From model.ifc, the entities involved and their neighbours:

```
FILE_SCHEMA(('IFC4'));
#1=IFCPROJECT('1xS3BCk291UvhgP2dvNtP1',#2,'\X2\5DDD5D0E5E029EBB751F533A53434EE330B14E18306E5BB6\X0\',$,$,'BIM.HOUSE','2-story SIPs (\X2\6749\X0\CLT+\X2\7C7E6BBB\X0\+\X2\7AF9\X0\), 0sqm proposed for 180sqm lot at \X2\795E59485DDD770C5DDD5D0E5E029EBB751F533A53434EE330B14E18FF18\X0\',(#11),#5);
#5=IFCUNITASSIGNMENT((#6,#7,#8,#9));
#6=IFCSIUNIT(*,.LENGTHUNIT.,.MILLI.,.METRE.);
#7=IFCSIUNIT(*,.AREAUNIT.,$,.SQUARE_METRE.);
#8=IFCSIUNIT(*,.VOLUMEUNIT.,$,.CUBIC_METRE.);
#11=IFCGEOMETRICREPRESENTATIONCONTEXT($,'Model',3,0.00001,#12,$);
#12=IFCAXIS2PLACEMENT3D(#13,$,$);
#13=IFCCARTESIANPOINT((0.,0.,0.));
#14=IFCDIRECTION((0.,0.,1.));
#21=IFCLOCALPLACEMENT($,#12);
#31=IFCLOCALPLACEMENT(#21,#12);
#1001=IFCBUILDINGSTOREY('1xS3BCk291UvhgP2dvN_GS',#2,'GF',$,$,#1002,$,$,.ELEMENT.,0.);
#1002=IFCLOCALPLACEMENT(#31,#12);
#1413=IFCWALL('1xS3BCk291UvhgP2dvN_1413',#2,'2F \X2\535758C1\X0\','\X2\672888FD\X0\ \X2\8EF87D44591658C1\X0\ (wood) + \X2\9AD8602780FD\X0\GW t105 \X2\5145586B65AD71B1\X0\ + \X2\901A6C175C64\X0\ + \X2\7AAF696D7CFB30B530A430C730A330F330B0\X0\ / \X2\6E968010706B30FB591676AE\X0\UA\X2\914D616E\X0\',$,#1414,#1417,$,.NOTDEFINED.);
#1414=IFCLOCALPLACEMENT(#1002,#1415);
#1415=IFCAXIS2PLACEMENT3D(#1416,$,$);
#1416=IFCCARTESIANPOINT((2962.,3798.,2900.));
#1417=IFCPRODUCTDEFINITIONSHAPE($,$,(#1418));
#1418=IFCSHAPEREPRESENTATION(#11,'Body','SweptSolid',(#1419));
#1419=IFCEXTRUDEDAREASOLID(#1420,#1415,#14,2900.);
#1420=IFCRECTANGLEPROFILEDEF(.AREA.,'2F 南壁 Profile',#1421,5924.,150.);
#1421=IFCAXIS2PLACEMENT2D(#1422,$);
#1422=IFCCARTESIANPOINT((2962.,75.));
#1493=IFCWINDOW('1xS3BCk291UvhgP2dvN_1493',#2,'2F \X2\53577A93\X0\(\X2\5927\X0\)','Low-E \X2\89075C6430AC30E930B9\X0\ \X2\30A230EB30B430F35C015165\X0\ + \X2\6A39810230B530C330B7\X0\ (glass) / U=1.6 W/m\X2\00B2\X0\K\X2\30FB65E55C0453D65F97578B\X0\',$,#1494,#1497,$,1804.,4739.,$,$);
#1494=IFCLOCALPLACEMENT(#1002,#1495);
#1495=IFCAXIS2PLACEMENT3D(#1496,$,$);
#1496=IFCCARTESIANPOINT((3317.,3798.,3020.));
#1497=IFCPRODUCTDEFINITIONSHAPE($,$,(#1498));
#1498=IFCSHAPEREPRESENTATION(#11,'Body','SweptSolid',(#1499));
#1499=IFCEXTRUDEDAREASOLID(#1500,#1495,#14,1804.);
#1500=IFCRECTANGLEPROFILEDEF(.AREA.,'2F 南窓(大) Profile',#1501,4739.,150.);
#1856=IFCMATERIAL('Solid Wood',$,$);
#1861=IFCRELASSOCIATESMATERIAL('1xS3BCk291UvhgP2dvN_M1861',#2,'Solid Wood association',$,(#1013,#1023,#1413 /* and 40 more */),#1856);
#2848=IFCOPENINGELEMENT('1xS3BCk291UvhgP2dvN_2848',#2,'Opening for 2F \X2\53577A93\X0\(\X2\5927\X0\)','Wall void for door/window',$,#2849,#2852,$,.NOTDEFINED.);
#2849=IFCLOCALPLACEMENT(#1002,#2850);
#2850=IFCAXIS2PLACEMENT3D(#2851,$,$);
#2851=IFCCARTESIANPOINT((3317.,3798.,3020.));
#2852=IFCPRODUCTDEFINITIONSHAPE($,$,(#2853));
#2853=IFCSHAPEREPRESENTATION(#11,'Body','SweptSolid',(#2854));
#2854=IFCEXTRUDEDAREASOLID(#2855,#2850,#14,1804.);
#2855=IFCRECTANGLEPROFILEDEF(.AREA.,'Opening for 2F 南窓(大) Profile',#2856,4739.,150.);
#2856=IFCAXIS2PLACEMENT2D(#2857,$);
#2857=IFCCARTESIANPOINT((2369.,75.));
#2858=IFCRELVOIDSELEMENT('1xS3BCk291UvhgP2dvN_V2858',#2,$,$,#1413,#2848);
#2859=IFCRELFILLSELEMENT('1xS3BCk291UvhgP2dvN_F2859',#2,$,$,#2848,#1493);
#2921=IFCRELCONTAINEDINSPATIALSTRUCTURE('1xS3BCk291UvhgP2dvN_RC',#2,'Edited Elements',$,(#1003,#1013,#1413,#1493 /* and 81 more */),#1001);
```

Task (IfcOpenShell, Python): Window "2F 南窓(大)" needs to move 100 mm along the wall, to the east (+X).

```python
import ifcopenshell
import ifcopenshell.api.geometry
import ifcopenshell.util.placement
import ifcopenshell.util.unit

model = ifcopenshell.open("model.ifc")
unit_scale = ifcopenshell.util.unit.calculate_unit_scale(model)

window = model.by_guid("1xS3BCk291UvhgP2dvN_1493")
opening = window.FillsVoids[0].RelatingOpeningElement
wall = opening.VoidsElements[0].RelatingBuildingElement

wall_matrix = ifcopenshell.util.placement.get_local_placement(wall.ObjectPlacement)
shift = wall_matrix[:3, 0] * 0.1 / unit_scale
before = ifcopenshell.util.placement.get_local_placement(window.ObjectPlacement)[:3, 3].copy()

# The window is not placed relative to its opening, so move both.
for product in (opening, window):
    matrix = ifcopenshell.util.placement.get_local_placement(product.ObjectPlacement)
    matrix[:3, 3] += shift
    ifcopenshell.api.geometry.edit_object_placement(model, product=product, matrix=matrix, is_si=False)

after = ifcopenshell.util.placement.get_local_placement(window.ObjectPlacement)[:3, 3]
print("window moved by", (after - before).round(3) + 0.0)

model.write("model-out.ifc")
```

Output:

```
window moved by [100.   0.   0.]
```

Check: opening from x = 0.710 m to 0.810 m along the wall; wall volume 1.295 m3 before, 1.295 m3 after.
